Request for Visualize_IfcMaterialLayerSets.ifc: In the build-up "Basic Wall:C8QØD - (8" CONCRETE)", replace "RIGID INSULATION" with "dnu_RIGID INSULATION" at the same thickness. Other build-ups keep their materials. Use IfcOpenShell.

First a look at what the model holds.

```python
import ifcopenshell
import ifcopenshell.util.element

model = ifcopenshell.open("Visualize_IfcMaterialLayerSets.ifc")
print(model.schema)
for layer_set in model.by_type("IfcMaterialLayerSet"):
    if layer_set.LayerSetName == 'Basic Wall:C8QØD - (8" CONCRETE)':
        for layer in layer_set.MaterialLayers:
            print(layer.id(), layer.Material and layer.Material.Name, layer.LayerThickness, sep=" | ")
        print(len(ifcopenshell.util.element.get_elements_by_material(model, layer_set)), "elements and types use it")
print(sorted(m.Name for m in model.by_type("IfcMaterial") if m.Name)[:60])
```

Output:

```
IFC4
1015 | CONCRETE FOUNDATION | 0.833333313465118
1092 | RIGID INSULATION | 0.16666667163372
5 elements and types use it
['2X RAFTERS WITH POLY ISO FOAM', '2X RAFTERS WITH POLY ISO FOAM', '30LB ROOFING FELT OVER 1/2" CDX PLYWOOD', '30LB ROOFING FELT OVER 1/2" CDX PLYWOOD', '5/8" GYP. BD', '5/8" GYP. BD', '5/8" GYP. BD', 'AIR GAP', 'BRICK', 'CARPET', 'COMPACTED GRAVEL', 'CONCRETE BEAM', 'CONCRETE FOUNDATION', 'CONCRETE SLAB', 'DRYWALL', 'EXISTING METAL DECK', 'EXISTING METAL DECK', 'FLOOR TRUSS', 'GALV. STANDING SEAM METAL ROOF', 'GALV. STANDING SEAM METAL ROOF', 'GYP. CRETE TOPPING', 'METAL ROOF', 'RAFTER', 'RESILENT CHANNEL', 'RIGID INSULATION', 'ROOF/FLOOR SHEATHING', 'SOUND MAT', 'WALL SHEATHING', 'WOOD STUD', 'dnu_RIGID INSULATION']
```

```python
import ifcopenshell
import ifcopenshell.api.material

model = ifcopenshell.open("Visualize_IfcMaterialLayerSets.ifc")

layer_set = next(s for s in model.by_type("IfcMaterialLayerSet") if s.LayerSetName == 'Basic Wall:C8QØD - (8" CONCRETE)')
layer = next(l for l in layer_set.MaterialLayers if l.Material and l.Material.Name == "RIGID INSULATION")
material = next(m for m in model.by_type("IfcMaterial") if m.Name == "dnu_RIGID INSULATION")

# Point this one layer at the other material; renaming the old one would change it everywhere.
ifcopenshell.api.material.edit_layer(model, layer=layer, attributes={}, material=material)

print([l.Material.Name if l.Material else None for l in layer_set.MaterialLayers])

model.write("Visualize_IfcMaterialLayerSets_v2.ifc")
```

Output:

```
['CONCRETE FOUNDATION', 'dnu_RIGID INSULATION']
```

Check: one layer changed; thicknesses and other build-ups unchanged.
